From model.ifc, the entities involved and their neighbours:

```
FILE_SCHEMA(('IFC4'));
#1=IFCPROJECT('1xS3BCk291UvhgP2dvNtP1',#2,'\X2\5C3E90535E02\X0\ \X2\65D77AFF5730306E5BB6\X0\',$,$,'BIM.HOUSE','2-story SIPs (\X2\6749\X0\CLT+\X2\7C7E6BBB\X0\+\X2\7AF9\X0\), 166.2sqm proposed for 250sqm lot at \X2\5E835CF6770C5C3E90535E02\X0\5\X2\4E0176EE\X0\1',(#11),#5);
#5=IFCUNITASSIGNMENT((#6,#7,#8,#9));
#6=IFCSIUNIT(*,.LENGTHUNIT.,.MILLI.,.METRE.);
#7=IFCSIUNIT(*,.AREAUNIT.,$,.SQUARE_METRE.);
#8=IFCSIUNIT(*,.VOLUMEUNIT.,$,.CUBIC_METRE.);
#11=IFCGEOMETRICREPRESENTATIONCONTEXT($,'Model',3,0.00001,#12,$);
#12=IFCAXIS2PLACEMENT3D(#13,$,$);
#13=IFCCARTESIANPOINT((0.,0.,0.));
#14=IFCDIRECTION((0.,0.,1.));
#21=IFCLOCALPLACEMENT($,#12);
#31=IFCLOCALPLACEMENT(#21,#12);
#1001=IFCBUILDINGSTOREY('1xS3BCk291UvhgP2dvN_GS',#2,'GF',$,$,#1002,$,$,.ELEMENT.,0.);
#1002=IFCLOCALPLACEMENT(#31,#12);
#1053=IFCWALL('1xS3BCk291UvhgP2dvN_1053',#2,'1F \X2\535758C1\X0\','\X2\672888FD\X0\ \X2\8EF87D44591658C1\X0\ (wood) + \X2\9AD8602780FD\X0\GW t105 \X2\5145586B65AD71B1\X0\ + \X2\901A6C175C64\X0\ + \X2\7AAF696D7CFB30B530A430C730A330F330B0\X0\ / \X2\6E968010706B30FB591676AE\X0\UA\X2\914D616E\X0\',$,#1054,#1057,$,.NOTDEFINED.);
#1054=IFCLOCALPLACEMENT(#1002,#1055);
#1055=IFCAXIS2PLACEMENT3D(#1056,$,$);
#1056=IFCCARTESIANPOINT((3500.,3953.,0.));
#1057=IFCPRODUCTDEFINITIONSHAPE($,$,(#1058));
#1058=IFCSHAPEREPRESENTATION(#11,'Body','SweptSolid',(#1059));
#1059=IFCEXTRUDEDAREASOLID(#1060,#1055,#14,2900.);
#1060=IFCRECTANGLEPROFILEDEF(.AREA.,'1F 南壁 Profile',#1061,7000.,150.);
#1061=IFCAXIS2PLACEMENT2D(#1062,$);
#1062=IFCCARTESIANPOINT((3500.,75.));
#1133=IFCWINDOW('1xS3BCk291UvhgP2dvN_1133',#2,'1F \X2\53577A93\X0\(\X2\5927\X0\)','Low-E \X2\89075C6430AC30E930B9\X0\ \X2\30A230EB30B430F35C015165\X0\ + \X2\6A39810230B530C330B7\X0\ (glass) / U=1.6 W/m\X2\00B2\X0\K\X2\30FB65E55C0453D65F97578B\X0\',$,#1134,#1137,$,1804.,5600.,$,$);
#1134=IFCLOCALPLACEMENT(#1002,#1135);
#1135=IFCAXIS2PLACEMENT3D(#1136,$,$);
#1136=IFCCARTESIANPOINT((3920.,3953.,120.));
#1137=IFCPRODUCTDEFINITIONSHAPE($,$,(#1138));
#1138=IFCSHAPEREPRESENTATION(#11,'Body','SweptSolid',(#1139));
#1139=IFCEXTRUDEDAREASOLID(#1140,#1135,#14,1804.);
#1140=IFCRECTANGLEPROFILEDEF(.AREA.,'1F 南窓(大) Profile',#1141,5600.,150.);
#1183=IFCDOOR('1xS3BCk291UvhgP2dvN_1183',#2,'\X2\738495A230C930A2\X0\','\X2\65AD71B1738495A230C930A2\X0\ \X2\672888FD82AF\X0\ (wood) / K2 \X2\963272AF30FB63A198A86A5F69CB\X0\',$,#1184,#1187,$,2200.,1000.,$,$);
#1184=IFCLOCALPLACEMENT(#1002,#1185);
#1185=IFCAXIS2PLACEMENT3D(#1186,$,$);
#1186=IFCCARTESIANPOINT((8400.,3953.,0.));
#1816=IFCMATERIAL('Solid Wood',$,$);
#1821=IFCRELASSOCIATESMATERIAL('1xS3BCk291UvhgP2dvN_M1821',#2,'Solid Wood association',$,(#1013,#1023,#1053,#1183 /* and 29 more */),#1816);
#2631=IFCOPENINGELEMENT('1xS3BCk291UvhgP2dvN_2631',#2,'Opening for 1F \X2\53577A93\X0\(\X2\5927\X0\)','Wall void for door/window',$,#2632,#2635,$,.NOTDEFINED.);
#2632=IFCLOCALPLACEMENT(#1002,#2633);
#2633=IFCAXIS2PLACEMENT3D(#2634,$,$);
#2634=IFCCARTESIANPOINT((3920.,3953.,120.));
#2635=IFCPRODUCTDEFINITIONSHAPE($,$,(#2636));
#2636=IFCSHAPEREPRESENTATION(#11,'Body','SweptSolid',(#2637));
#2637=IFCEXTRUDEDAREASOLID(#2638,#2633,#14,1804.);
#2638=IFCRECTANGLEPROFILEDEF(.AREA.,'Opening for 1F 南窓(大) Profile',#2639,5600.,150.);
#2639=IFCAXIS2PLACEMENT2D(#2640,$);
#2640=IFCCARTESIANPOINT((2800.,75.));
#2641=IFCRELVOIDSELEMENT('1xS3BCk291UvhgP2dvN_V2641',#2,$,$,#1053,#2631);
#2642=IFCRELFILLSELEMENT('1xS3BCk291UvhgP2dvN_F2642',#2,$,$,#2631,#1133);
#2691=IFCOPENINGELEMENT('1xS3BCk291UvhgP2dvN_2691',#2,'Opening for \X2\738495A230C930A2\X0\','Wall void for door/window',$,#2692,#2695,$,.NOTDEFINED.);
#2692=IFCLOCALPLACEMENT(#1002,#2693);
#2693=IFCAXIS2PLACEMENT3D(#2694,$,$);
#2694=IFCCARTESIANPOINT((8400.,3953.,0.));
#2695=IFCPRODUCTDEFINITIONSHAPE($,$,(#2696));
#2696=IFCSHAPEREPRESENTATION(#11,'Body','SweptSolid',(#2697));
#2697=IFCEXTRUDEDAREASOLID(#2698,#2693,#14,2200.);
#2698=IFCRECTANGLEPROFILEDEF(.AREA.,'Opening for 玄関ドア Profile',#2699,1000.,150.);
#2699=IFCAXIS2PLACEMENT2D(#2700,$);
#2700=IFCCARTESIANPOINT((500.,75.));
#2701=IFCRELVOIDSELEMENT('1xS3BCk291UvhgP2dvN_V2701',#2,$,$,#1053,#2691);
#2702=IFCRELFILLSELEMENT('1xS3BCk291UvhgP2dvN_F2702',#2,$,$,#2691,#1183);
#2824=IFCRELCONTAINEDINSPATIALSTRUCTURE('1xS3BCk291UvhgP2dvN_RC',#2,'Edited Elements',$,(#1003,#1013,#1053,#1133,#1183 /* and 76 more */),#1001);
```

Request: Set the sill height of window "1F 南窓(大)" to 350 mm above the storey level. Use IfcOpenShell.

```python
import numpy as np
import ifcopenshell
import ifcopenshell.api.geometry
import ifcopenshell.geom
import ifcopenshell.util.element
import ifcopenshell.util.placement
import ifcopenshell.util.shape
import ifcopenshell.util.unit

model = ifcopenshell.open("model.ifc")
unit_scale = ifcopenshell.util.unit.calculate_unit_scale(model)

window = model.by_guid("1xS3BCk291UvhgP2dvN_1133")
opening = window.FillsVoids[0].RelatingOpeningElement
storey = ifcopenshell.util.element.get_container(window, ifc_class="IfcBuildingStorey")
level = ifcopenshell.util.placement.get_local_placement(storey.ObjectPlacement)[2, 3]

# The opening's origin need not be at the sill, so measure its lowest point.
shape = ifcopenshell.geom.create_shape(ifcopenshell.geom.settings(), opening)
bottom = ifcopenshell.util.shape.get_shape_bottom_elevation(shape, shape.geometry) / unit_scale
dz = level + 0.35 / unit_scale - bottom

shift = np.array([0.0, 0.0, dz])
# The window is not placed relative to its opening, so move both.
for product in (opening, window):
    matrix = ifcopenshell.util.placement.get_local_placement(product.ObjectPlacement)
    matrix[:3, 3] += shift
    ifcopenshell.api.geometry.edit_object_placement(model, product=product, matrix=matrix, is_si=False)

print(f"moved by {dz * unit_scale:+.3f} m")

model.write("model_v2.ifc")
```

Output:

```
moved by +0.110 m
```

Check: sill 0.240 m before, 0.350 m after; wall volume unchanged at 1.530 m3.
